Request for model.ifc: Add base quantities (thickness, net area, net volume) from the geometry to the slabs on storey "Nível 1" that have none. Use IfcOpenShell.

First a look at what the model holds.

```python
import ifcopenshell
import ifcopenshell.util.element
import ifcopenshell.util.unit

model = ifcopenshell.open("model.ifc")
print(model.schema)
for unit_type in ("LENGTHUNIT", "AREAUNIT", "VOLUMEUNIT"):
    print(unit_type, ifcopenshell.util.unit.calculate_unit_scale(model, unit_type))
storey = next(s for s in model.by_type("IfcBuildingStorey") if s.Name == "Nível 1")
slabs = [e for e in ifcopenshell.util.element.get_decomposition(storey) if e.is_a("IfcSlab")]
for e in sorted(slabs, key=lambda e: e.id()):
    print(e.id(), e.is_a(), e.Name, list(ifcopenshell.util.element.get_psets(e, qtos_only=True)), sep=" | ")
```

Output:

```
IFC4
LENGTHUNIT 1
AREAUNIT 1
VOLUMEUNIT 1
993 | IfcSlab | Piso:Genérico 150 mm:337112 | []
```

```python
import ifcopenshell
import ifcopenshell.api.pset
import ifcopenshell.geom
import ifcopenshell.util.element
import ifcopenshell.util.shape
import ifcopenshell.util.unit

model = ifcopenshell.open("model.ifc")
unit_scale = ifcopenshell.util.unit.calculate_unit_scale(model)
area_scale = ifcopenshell.util.unit.calculate_unit_scale(model, "AREAUNIT")
volume_scale = ifcopenshell.util.unit.calculate_unit_scale(model, "VOLUMEUNIT")
settings = ifcopenshell.geom.settings()

storey = next(s for s in model.by_type("IfcBuildingStorey") if s.Name == "Nível 1")
slabs = [e for e in ifcopenshell.util.element.get_decomposition(storey) if e.is_a("IfcSlab")]

for e in sorted(slabs, key=lambda e: e.id()):
    if ifcopenshell.util.element.get_psets(e, qtos_only=True, should_inherit=False):
        continue
    # Geometry comes back in metres, in the element's own axes.
    shape = ifcopenshell.geom.create_shape(settings, e)
    values = {
        "Width": ifcopenshell.util.shape.get_z(shape.geometry) / unit_scale,
        "NetArea": ifcopenshell.util.shape.get_footprint_area(shape.geometry) / area_scale,
        "NetVolume": ifcopenshell.util.shape.get_volume(shape.geometry) / volume_scale,
    }
    qto = ifcopenshell.api.pset.add_qto(model, product=e, name="Qto_SlabBaseQuantities")
    ifcopenshell.api.pset.edit_qto(model, qto=qto, properties=values)
    print(e.id(), {k: round(v, 3) for k, v in values.items()})

model.write("model-out.ifc")
```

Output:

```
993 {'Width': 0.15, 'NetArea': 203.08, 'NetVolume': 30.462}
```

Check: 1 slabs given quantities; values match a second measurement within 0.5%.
